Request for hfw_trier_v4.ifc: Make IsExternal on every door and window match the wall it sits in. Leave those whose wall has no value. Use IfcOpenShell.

First a look at what the model holds.

```python
import ifcopenshell
import ifcopenshell.util.element

model = ifcopenshell.open("hfw_trier_v4.ifc")
print(model.schema)
seen = {}
for e in model.by_type("IfcDoor") + model.by_type("IfcWindow"):
    if not e.FillsVoids:
        continue
    host = e.FillsVoids[0].RelatingOpeningElement.VoidsElements[0].RelatingBuildingElement
    own = ifcopenshell.util.element.get_pset(e, f"Pset_{e.is_a()[3:].removesuffix('StandardCase')}Common", "IsExternal")
    wall = ifcopenshell.util.element.get_pset(host, "Pset_WallCommon", "IsExternal")
    seen[e.is_a(), own, wall] = seen.get((e.is_a(), own, wall), 0) + 1
for (cls, own, wall), count in sorted(seen.items(), key=str):
    print(count, cls, "IsExternal:", own, "| host wall:", wall)
```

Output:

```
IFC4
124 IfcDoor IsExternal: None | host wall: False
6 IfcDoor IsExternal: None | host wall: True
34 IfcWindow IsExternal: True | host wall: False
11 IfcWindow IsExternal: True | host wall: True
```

```python
import ifcopenshell
import ifcopenshell.api.pset
import ifcopenshell.util.element

model = ifcopenshell.open("hfw_trier_v4.ifc")

count = 0
for ifc_class, pset_name in (("IfcDoor", "Pset_DoorCommon"), ("IfcWindow", "Pset_WindowCommon")):
    for e in model.by_type(ifc_class):
        if not e.FillsVoids:
            continue
        host = e.FillsVoids[0].RelatingOpeningElement.VoidsElements[0].RelatingBuildingElement
        external = ifcopenshell.util.element.get_pset(host, "Pset_WallCommon", "IsExternal")
        if external is None or ifcopenshell.util.element.get_pset(e, pset_name, "IsExternal") == external:
            continue
        pset = ifcopenshell.api.pset.add_pset(model, product=e, name=pset_name)
        ifcopenshell.api.pset.edit_pset(model, pset=pset, properties={"IsExternal": external})
        count += 1

print(count, "updated")

model.write("hfw_trier_v4_edited.ifc")
```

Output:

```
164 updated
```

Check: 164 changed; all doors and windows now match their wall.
